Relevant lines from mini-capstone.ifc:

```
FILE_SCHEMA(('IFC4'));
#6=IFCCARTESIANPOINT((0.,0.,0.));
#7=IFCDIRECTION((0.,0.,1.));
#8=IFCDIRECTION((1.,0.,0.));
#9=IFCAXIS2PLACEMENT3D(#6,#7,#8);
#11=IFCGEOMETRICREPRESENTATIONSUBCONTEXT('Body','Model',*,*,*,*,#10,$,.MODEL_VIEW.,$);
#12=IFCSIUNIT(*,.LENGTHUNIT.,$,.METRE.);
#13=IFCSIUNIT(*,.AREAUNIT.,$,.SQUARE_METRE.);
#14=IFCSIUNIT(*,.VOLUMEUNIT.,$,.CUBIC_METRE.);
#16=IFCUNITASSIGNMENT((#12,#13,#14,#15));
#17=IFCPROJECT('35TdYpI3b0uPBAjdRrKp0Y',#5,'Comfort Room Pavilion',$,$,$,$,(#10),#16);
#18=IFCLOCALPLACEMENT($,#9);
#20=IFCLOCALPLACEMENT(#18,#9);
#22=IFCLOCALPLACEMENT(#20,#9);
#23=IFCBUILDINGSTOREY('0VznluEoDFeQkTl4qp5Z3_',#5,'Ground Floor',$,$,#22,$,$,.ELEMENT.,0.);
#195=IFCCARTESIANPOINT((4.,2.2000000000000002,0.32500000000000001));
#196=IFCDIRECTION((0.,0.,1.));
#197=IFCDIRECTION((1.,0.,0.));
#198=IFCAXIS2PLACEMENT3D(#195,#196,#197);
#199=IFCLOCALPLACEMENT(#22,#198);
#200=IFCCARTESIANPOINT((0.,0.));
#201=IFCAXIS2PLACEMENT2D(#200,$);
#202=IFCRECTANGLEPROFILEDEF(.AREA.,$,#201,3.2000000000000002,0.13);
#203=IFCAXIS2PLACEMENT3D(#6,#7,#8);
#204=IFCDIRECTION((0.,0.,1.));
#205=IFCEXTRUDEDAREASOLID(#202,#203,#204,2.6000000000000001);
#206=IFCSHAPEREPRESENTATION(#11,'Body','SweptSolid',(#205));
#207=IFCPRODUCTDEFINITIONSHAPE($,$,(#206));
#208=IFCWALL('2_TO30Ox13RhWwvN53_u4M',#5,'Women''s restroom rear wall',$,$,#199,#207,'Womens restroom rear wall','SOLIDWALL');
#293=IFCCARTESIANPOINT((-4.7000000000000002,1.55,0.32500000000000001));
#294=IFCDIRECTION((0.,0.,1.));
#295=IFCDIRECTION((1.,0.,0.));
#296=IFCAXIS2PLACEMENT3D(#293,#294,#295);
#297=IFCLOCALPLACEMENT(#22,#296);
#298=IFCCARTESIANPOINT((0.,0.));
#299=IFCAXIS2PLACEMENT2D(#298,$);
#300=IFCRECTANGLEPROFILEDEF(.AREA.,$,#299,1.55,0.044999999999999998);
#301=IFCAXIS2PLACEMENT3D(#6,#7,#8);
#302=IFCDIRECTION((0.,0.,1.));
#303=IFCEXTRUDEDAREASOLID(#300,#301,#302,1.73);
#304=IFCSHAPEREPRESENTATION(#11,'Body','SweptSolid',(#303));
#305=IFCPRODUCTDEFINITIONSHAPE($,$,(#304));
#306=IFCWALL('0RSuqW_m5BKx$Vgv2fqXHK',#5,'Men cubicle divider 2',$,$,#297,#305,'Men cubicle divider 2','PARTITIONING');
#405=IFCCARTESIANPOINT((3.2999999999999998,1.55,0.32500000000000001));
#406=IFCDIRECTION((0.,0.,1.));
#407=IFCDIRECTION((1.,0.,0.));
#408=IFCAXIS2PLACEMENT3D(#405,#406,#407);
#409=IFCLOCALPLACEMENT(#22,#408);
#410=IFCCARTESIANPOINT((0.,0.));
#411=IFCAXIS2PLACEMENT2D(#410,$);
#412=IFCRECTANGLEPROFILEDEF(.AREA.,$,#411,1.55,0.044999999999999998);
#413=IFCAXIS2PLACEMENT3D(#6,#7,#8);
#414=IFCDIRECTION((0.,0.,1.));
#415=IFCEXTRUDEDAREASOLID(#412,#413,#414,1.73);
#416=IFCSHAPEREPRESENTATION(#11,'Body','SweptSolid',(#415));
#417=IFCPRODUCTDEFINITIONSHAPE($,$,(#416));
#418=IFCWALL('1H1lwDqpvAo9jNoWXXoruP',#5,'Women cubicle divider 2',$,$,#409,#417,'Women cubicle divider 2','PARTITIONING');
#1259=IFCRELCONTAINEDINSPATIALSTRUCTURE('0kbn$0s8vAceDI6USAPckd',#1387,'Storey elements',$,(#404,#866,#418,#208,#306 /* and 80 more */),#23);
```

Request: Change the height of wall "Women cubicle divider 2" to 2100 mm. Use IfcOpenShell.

```python
import ifcopenshell
import ifcopenshell.geom
import ifcopenshell.util.representation
import ifcopenshell.util.shape

model = ifcopenshell.open("mini-capstone.ifc")
settings = ifcopenshell.geom.settings()


def volume(element):
    """Net volume in cubic metres, openings subtracted."""
    shape = ifcopenshell.geom.create_shape(settings, element)
    return ifcopenshell.util.shape.get_volume(shape.geometry)


wall = model.by_guid("1H1lwDqpvAo9jNoWXXoruP")
before = volume(wall)

body = ifcopenshell.util.representation.get_representation(wall, "Model", "Body")
solid = body.Items[0]
old_height = solid.Depth
solid.Depth = 2.1
after = volume(wall)

print(f"height {old_height:g} -> {solid.Depth:g}, volume {before:.3f} -> {after:.3f} m3")

model.write("mini-capstone_v2.ifc")
```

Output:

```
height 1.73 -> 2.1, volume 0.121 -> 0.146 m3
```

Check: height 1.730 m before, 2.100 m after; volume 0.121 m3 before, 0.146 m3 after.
